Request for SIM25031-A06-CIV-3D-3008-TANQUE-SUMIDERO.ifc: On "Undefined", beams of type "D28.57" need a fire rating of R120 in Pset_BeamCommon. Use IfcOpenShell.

First a look at what the model holds.

```python
import ifcopenshell
import ifcopenshell.util.element

model = ifcopenshell.open("SIM25031-A06-CIV-3D-3008-TANQUE-SUMIDERO.ifc")
print(model.schema)
storey = next(s for s in model.by_type("IfcBuildingStorey") if s.Name == "Undefined")
beams = [e for e in ifcopenshell.util.element.get_decomposition(storey) if e.is_a("IfcBeam")]
seen = {}
for e in beams:
    element_type = ifcopenshell.util.element.get_type(e)
    key = (element_type.Name if element_type != e and element_type else None, ifcopenshell.util.element.get_pset(e, "Pset_BeamCommon", "FireRating"))
    seen[key] = seen.get(key, 0) + 1
for (name, value), count in sorted(seen.items(), key=str):
    print(count, "x", name, "|", value)
```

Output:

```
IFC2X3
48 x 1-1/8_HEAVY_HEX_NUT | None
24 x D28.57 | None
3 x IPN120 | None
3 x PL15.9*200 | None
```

```python
import ifcopenshell
import ifcopenshell.api.pset
import ifcopenshell.util.element

model = ifcopenshell.open("SIM25031-A06-CIV-3D-3008-TANQUE-SUMIDERO.ifc")

storey = next(s for s in model.by_type("IfcBuildingStorey") if s.Name == "Undefined")
beams = [e for e in ifcopenshell.util.element.get_decomposition(storey) if e.is_a("IfcBeam")]

count = 0
for e in beams:
    element_type = ifcopenshell.util.element.get_type(e)
    if element_type in (None, e) or element_type.Name != "D28.57":
        continue
    found = ifcopenshell.util.element.get_pset(e, "Pset_BeamCommon", should_inherit=False)
    if found:
        pset = model.by_id(found["id"])
        if len(ifcopenshell.util.element.get_elements_by_pset(pset)) > 1:
            pset = ifcopenshell.api.pset.unshare_pset(model, products=[e], pset=pset)[0]
    else:
        pset = ifcopenshell.api.pset.add_pset(model, product=e, name="Pset_BeamCommon")
    ifcopenshell.api.pset.edit_pset(model, pset=pset, properties={"FireRating": "R120"})
    count += 1

print(count, "beams updated")

model.write("SIM25031-A06-CIV-3D-3008-TANQUE-SUMIDERO_edited.ifc")
```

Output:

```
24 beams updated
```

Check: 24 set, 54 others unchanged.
